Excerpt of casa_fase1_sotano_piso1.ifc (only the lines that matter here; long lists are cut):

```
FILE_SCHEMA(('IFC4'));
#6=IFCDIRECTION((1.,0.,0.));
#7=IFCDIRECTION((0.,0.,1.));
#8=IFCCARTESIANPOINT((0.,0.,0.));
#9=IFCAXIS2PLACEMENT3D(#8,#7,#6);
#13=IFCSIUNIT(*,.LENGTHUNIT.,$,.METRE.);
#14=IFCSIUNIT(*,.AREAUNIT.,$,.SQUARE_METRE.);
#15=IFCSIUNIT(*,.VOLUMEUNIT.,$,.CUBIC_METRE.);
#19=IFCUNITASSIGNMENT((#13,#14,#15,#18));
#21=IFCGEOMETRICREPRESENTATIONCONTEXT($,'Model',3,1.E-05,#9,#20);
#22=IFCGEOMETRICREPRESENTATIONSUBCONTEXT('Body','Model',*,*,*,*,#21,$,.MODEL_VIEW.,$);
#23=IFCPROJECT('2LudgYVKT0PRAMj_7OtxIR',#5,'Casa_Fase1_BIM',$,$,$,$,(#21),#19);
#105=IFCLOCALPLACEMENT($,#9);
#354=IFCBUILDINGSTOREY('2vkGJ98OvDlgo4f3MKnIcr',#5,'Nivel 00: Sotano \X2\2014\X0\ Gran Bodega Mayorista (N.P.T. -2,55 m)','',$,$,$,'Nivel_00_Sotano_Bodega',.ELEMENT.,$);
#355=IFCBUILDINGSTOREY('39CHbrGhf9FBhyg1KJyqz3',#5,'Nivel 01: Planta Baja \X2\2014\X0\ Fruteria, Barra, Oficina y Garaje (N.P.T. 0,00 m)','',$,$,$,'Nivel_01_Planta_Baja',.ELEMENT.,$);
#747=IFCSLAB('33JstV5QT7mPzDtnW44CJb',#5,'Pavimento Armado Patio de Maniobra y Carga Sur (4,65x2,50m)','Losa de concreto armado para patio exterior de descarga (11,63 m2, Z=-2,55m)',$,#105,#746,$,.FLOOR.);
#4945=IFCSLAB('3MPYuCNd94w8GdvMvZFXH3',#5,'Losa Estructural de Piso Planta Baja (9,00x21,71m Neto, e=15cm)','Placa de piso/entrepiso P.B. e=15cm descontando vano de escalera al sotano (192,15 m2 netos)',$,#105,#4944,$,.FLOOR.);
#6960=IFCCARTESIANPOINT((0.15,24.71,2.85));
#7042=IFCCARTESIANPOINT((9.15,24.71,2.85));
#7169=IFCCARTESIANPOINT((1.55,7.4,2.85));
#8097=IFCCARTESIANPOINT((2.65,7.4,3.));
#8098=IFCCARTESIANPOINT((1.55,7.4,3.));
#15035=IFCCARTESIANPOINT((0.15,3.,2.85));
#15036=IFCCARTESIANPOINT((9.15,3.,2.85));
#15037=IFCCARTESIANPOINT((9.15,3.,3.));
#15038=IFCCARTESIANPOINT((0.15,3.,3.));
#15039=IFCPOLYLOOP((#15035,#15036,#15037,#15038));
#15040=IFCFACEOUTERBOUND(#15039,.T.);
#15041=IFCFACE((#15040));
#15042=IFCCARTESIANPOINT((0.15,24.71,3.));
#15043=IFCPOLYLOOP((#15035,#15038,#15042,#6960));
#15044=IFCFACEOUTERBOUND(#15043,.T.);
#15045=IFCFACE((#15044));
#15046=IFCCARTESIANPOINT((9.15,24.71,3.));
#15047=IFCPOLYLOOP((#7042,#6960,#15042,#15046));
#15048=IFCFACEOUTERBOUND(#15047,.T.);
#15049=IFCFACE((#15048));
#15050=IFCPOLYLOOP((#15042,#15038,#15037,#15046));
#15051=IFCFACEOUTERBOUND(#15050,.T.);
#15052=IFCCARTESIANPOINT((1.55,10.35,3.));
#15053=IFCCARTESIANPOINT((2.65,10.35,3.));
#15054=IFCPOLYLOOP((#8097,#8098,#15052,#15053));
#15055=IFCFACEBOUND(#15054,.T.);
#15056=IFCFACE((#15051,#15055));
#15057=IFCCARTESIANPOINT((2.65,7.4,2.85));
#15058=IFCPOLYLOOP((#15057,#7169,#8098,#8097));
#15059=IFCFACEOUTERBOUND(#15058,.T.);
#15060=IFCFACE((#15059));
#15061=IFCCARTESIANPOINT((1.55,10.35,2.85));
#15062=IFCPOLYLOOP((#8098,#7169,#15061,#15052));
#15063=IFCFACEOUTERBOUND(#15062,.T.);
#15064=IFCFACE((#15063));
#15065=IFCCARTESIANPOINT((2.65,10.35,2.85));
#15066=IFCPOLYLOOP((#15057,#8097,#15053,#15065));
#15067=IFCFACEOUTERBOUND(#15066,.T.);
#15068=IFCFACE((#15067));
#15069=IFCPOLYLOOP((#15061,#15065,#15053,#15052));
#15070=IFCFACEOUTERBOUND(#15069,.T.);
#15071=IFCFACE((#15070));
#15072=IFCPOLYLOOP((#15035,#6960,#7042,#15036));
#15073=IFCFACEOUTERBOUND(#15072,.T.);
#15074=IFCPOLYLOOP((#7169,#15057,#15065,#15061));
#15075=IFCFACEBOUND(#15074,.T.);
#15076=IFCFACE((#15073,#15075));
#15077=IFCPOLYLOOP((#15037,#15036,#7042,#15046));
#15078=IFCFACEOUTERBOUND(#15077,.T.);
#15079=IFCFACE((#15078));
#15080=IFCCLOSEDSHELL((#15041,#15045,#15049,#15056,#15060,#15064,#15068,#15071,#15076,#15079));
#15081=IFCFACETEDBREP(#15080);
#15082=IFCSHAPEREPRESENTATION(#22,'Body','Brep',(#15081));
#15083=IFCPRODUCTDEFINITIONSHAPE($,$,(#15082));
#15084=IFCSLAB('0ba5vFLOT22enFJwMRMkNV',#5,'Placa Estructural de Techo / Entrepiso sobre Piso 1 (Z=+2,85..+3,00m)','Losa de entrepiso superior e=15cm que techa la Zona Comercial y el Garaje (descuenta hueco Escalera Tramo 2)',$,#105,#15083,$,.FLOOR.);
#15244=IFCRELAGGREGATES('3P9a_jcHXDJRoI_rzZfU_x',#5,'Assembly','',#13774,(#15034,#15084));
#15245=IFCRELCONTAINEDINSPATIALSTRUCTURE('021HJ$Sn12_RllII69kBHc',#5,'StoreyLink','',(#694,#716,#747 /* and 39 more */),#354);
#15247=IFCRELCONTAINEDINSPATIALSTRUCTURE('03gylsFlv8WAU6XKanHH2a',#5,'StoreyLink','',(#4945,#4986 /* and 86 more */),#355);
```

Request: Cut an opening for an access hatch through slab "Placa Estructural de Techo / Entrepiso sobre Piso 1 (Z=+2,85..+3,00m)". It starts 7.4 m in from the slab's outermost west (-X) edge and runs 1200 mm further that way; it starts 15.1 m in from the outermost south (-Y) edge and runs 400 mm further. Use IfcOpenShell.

```python
import numpy as np
import ifcopenshell
import ifcopenshell.api.feature
import ifcopenshell.api.geometry
import ifcopenshell.api.root
import ifcopenshell.geom
import ifcopenshell.util.placement
import ifcopenshell.util.representation
import ifcopenshell.util.shape
import ifcopenshell.util.unit

model = ifcopenshell.open("casa_fase1_sotano_piso1.ifc")
unit_scale = ifcopenshell.util.unit.calculate_unit_scale(model)
settings = ifcopenshell.geom.settings()


def volume(element):
    """Net volume in cubic metres, openings subtracted."""
    shape = ifcopenshell.geom.create_shape(settings, element)
    return ifcopenshell.util.shape.get_volume(shape.geometry)


slab = model.by_id(15084)
before = volume(slab)

# Extent in the slab's own axes, in metres. The edges named are its -X and -Y sides.
slab_shape = ifcopenshell.geom.create_shape(settings, slab)
vertices = ifcopenshell.util.shape.get_vertices(slab_shape.geometry)
x_min, y_min, bottom = vertices.min(axis=0)
top = vertices[:, 2].max()

opening = ifcopenshell.api.root.create_entity(model, ifc_class="IfcOpeningElement", name="Access hatch opening", predefined_type="OPENING")
context = ifcopenshell.util.representation.get_context(model, "Model", "Body", "MODEL_VIEW")
width, depth = 1.2, 0.4
outline = [(0.0, 0.0), (width, 0.0), (width, depth), (0.0, depth), (0.0, 0.0)]
# Overshoot both faces by 50 mm so the cut is clean.
shape = ifcopenshell.api.geometry.add_slab_representation(
    model, context=context, depth=top - bottom + 0.1, polyline=outline
)
ifcopenshell.api.geometry.assign_representation(model, product=opening, representation=shape)

matrix = ifcopenshell.util.placement.get_local_placement(slab.ObjectPlacement)
matrix[:, 3] = matrix @ np.append(np.array([x_min + 7.4, y_min + 15.1, bottom - 0.05]) / unit_scale, 1.0)
ifcopenshell.api.geometry.edit_object_placement(model, product=opening, matrix=matrix, is_si=False)
ifcopenshell.api.feature.add_feature(model, feature=opening, element=slab)

after = volume(slab)

print(f"slab volume {before:.3f} -> {after:.3f} m3")

model.write("casa_fase1_sotano_piso1_rev.ifc")
```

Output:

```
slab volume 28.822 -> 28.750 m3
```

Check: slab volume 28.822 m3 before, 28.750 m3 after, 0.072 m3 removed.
